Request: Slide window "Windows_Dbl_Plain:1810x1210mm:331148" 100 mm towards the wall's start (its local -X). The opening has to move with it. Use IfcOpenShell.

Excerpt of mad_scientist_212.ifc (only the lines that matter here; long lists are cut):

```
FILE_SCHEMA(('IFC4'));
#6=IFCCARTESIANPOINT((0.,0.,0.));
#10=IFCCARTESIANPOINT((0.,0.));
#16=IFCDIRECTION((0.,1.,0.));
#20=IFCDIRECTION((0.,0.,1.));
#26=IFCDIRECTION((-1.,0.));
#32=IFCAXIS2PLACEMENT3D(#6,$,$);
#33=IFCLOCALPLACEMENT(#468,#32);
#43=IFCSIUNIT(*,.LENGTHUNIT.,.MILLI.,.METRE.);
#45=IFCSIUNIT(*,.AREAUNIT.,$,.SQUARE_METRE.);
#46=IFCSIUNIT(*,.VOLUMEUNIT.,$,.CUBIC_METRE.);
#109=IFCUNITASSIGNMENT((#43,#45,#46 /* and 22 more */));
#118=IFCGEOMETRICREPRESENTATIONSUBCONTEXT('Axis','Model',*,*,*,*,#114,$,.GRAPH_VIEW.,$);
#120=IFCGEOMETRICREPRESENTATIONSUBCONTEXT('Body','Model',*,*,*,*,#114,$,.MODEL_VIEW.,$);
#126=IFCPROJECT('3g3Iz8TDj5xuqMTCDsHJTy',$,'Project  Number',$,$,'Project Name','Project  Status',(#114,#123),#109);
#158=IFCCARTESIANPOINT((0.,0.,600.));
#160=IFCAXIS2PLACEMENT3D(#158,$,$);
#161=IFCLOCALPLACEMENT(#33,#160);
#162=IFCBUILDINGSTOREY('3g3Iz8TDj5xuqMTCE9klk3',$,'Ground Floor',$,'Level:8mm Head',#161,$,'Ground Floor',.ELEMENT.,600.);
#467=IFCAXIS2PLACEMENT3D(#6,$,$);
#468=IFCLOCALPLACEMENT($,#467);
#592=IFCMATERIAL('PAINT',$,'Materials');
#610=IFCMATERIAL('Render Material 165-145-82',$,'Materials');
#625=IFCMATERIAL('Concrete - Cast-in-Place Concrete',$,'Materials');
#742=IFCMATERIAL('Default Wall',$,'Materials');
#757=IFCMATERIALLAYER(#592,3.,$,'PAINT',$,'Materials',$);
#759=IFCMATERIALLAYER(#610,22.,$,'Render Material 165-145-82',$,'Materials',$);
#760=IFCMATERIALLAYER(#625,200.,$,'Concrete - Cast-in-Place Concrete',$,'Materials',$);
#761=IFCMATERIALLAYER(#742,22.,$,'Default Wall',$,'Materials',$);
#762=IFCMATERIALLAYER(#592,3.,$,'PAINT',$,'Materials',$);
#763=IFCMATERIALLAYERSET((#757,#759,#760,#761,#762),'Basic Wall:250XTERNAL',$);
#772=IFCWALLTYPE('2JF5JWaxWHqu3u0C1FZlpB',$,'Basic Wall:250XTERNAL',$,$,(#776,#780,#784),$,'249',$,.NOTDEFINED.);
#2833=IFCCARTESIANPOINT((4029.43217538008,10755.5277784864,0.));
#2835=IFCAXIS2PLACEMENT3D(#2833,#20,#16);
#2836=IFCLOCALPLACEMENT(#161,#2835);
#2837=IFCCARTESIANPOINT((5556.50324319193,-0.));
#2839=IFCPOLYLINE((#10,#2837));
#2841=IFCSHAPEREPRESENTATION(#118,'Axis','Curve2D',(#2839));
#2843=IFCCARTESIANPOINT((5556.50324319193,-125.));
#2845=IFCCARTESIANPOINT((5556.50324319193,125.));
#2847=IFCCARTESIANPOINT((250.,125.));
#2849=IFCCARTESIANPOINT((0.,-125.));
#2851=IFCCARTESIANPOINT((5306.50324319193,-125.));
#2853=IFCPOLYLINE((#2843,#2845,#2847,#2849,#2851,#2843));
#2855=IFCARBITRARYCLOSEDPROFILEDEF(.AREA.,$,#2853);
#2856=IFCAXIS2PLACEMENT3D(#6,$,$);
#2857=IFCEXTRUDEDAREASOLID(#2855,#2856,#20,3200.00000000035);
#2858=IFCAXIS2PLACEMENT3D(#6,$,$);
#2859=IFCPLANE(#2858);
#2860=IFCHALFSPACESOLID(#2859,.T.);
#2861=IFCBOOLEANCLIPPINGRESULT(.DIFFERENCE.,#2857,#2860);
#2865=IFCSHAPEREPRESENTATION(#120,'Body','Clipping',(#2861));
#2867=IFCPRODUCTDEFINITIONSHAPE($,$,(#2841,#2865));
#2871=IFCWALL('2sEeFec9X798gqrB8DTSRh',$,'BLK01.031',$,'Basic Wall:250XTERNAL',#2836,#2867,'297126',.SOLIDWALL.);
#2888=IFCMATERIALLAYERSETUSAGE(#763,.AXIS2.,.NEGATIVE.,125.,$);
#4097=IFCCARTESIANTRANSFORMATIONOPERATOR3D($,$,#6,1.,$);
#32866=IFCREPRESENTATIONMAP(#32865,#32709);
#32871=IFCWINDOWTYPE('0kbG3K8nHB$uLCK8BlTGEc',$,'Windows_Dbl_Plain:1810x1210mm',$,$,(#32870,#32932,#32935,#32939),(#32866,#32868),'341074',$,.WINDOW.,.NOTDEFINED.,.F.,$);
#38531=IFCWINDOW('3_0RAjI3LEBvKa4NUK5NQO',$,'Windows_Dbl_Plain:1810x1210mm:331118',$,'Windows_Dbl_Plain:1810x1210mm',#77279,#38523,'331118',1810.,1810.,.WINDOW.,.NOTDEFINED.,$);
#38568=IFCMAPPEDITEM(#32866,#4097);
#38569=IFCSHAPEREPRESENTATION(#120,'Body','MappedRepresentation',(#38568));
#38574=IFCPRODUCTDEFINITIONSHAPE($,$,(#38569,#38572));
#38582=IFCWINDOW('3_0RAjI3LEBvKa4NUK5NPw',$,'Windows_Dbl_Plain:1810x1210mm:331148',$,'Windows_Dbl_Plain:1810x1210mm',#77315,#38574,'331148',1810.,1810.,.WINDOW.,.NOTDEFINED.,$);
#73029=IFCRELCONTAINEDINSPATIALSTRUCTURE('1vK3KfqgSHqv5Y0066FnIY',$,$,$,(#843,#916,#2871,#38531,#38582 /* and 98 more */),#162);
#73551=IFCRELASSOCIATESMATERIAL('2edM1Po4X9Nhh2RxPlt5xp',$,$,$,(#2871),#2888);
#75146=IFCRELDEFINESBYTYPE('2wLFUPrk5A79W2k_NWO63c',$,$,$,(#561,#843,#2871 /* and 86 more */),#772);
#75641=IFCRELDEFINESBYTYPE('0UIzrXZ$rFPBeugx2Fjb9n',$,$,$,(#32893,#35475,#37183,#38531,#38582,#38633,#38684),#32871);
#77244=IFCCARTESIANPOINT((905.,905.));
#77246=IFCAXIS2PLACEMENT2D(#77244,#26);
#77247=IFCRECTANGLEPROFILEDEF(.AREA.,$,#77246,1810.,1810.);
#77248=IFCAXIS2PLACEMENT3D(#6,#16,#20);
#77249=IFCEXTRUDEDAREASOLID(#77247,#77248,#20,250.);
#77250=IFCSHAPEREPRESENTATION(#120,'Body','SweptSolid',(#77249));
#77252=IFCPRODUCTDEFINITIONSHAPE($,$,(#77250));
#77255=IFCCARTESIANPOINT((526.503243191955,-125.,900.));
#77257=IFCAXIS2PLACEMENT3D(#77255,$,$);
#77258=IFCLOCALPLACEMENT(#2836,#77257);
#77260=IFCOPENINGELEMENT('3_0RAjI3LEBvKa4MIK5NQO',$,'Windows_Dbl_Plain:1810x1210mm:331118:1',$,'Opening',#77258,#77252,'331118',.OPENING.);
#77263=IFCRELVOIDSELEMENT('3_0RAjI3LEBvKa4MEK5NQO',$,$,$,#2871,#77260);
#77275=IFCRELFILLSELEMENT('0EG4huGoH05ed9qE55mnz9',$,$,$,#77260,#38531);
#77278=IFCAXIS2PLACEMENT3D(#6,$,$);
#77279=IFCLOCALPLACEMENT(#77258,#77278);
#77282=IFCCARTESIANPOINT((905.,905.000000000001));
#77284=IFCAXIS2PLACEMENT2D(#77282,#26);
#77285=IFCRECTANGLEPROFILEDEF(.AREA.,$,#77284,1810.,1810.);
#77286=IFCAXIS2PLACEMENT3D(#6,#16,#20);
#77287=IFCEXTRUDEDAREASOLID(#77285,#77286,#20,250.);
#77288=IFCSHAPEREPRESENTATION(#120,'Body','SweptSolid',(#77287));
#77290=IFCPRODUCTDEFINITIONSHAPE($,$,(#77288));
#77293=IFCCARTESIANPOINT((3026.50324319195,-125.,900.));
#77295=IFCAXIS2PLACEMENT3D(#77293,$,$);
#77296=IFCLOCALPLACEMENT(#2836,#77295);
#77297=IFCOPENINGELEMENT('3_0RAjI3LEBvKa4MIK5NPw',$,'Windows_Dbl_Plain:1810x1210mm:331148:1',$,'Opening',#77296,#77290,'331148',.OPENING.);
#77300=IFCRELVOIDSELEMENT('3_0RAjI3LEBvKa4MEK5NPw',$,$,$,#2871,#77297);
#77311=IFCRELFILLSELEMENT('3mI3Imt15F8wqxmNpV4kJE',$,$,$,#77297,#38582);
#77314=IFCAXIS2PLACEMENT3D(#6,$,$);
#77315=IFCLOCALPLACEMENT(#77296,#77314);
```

```python
import ifcopenshell
import ifcopenshell.api.geometry
import ifcopenshell.util.placement
import ifcopenshell.util.unit

model = ifcopenshell.open("mad_scientist_212.ifc")
unit_scale = ifcopenshell.util.unit.calculate_unit_scale(model)

window = model.by_guid("3_0RAjI3LEBvKa4NUK5NPw")
opening = window.FillsVoids[0].RelatingOpeningElement
wall = opening.VoidsElements[0].RelatingBuildingElement

wall_matrix = ifcopenshell.util.placement.get_local_placement(wall.ObjectPlacement)
shift = wall_matrix[:3, 0] * -0.1 / unit_scale
before = ifcopenshell.util.placement.get_local_placement(window.ObjectPlacement)[:3, 3].copy()

# The window is placed relative to its opening, so it follows when the opening moves.
matrix = ifcopenshell.util.placement.get_local_placement(opening.ObjectPlacement)
matrix[:3, 3] += shift
ifcopenshell.api.geometry.edit_object_placement(
    model, product=opening, matrix=matrix, is_si=False, should_transform_children=True
)

after = ifcopenshell.util.placement.get_local_placement(window.ObjectPlacement)[:3, 3]
print("window moved by", (after - before).round(3) + 0.0)

model.write("mad_scientist_212_v2.ifc")
```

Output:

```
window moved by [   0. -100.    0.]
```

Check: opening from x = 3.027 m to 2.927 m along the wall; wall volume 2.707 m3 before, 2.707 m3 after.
